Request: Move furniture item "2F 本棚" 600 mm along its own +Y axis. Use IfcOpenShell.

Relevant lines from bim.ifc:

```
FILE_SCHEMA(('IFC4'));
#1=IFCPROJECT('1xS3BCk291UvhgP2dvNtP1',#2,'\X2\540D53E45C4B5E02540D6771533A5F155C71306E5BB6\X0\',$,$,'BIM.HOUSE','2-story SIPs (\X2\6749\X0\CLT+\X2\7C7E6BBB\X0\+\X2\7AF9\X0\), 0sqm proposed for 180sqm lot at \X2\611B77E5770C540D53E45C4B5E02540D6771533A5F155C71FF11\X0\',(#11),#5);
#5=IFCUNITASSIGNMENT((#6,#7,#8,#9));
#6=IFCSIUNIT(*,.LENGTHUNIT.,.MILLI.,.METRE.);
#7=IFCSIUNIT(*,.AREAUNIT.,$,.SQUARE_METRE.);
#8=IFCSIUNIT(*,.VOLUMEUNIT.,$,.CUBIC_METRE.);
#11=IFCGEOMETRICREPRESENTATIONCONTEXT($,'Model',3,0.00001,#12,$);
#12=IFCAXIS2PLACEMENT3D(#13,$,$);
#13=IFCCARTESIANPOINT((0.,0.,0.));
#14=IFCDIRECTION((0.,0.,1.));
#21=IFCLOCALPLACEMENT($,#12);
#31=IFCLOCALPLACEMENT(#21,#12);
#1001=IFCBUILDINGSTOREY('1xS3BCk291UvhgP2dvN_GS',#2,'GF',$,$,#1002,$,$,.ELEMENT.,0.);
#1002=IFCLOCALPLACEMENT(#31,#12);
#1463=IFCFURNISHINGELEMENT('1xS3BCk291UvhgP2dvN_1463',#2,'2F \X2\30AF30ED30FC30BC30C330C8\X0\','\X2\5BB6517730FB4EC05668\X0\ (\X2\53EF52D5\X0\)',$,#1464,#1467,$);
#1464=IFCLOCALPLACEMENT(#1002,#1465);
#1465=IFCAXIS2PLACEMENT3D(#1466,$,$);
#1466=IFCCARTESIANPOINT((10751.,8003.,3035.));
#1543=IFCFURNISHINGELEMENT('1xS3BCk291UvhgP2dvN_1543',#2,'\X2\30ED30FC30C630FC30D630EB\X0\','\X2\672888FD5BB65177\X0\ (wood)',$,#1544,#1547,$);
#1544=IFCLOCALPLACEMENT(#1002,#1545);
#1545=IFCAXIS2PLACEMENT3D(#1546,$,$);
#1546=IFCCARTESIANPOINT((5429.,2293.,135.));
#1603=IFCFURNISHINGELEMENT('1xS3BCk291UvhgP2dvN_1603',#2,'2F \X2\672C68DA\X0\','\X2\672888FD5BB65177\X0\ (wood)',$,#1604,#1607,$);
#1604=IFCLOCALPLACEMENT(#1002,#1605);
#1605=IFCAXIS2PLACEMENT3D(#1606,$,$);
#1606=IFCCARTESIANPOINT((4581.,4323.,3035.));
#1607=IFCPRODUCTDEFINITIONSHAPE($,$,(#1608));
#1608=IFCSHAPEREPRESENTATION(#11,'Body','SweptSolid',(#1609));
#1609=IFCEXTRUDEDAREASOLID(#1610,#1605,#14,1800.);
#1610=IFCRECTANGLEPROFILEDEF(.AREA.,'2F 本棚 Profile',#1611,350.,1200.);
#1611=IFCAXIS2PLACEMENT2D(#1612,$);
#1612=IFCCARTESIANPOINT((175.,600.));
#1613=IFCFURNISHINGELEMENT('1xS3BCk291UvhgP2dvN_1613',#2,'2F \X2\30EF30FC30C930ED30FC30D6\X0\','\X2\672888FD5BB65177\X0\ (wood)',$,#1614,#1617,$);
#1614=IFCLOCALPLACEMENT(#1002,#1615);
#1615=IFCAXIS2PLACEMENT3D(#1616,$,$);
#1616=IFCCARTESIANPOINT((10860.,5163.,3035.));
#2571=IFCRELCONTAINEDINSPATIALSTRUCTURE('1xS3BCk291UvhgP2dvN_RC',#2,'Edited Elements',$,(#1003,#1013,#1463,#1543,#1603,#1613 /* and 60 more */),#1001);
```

```python
import ifcopenshell
import ifcopenshell.api.geometry
import ifcopenshell.util.placement

model = ifcopenshell.open("bim.ifc")

item = model.by_id(1603)
matrix = ifcopenshell.util.placement.get_local_placement(item.ObjectPlacement)
matrix[:3, 3] += matrix[:3, 1] * 600.0
ifcopenshell.api.geometry.edit_object_placement(model, product=item, matrix=matrix, is_si=False)

print(ifcopenshell.util.placement.get_local_placement(item.ObjectPlacement).round(3) + 0.0)

model.write("bim_rev.ifc")
```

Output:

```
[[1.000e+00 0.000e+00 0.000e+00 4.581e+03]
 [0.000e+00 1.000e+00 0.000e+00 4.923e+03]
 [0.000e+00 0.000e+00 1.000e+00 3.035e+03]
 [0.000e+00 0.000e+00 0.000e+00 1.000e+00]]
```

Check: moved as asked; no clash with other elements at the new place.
